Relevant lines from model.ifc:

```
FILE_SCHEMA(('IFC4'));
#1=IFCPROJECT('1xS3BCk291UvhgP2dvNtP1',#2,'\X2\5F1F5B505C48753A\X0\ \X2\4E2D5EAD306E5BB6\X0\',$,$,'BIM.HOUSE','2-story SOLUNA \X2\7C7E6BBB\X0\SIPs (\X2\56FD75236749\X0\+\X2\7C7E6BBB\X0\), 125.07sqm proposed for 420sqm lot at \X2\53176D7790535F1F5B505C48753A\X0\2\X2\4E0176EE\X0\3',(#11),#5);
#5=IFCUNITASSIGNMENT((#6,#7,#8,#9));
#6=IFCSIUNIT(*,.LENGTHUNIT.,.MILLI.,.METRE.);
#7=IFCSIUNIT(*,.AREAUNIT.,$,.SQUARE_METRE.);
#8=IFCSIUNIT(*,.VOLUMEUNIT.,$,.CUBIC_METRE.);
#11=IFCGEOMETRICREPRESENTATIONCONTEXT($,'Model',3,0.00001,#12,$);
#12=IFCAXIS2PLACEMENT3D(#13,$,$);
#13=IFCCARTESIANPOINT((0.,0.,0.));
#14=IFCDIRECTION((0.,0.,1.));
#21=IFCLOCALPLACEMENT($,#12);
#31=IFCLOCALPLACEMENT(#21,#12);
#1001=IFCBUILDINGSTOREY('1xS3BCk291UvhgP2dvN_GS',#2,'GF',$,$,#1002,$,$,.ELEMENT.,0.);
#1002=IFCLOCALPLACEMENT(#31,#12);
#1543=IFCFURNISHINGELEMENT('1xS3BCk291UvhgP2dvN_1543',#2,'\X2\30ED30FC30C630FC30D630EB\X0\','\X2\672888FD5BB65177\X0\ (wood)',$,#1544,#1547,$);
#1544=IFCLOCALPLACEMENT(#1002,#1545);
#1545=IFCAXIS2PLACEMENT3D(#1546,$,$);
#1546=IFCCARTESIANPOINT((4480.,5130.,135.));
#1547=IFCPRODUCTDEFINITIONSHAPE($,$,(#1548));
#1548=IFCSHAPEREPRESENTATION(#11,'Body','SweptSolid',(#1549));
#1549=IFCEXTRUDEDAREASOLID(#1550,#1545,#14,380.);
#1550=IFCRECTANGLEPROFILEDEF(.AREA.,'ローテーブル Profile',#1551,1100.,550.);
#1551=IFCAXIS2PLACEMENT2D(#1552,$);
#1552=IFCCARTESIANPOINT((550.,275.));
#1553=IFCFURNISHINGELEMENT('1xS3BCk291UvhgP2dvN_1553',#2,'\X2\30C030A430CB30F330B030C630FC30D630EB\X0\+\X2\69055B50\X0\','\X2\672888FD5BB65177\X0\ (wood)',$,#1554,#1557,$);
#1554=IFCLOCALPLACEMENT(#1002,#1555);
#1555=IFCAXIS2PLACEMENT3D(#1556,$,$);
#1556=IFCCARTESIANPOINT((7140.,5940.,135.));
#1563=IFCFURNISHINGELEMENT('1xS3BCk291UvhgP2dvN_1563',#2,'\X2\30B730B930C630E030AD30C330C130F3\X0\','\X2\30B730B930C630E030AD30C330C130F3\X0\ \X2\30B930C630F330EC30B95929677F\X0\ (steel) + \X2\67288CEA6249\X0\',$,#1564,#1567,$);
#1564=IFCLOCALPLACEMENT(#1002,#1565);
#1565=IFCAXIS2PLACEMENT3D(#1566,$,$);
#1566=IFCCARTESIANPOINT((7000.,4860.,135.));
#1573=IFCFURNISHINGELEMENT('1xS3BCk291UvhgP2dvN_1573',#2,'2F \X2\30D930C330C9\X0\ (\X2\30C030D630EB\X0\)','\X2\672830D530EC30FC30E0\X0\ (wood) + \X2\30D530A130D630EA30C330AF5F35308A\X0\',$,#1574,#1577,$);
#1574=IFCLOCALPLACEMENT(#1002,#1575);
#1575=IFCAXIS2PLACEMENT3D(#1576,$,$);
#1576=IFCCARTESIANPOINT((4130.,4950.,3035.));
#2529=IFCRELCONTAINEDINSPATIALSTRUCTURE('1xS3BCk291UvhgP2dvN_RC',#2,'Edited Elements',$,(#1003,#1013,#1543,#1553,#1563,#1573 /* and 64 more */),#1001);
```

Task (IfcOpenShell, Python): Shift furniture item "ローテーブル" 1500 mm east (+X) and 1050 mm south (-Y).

```python
import ifcopenshell
import ifcopenshell.api.geometry
import ifcopenshell.util.placement

model = ifcopenshell.open("model.ifc")

item = model.by_guid("1xS3BCk291UvhgP2dvN_1543")
matrix = ifcopenshell.util.placement.get_local_placement(item.ObjectPlacement)
matrix[0, 3] += 1500.0
matrix[1, 3] -= 1050.0
ifcopenshell.api.geometry.edit_object_placement(model, product=item, matrix=matrix, is_si=False)

print(ifcopenshell.util.placement.get_local_placement(item.ObjectPlacement).round(3) + 0.0)

model.write("model_edited.ifc")
```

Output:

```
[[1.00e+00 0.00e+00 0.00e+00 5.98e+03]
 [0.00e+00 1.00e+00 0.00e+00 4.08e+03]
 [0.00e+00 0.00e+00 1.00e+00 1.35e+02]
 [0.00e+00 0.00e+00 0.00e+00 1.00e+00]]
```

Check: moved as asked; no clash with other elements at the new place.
